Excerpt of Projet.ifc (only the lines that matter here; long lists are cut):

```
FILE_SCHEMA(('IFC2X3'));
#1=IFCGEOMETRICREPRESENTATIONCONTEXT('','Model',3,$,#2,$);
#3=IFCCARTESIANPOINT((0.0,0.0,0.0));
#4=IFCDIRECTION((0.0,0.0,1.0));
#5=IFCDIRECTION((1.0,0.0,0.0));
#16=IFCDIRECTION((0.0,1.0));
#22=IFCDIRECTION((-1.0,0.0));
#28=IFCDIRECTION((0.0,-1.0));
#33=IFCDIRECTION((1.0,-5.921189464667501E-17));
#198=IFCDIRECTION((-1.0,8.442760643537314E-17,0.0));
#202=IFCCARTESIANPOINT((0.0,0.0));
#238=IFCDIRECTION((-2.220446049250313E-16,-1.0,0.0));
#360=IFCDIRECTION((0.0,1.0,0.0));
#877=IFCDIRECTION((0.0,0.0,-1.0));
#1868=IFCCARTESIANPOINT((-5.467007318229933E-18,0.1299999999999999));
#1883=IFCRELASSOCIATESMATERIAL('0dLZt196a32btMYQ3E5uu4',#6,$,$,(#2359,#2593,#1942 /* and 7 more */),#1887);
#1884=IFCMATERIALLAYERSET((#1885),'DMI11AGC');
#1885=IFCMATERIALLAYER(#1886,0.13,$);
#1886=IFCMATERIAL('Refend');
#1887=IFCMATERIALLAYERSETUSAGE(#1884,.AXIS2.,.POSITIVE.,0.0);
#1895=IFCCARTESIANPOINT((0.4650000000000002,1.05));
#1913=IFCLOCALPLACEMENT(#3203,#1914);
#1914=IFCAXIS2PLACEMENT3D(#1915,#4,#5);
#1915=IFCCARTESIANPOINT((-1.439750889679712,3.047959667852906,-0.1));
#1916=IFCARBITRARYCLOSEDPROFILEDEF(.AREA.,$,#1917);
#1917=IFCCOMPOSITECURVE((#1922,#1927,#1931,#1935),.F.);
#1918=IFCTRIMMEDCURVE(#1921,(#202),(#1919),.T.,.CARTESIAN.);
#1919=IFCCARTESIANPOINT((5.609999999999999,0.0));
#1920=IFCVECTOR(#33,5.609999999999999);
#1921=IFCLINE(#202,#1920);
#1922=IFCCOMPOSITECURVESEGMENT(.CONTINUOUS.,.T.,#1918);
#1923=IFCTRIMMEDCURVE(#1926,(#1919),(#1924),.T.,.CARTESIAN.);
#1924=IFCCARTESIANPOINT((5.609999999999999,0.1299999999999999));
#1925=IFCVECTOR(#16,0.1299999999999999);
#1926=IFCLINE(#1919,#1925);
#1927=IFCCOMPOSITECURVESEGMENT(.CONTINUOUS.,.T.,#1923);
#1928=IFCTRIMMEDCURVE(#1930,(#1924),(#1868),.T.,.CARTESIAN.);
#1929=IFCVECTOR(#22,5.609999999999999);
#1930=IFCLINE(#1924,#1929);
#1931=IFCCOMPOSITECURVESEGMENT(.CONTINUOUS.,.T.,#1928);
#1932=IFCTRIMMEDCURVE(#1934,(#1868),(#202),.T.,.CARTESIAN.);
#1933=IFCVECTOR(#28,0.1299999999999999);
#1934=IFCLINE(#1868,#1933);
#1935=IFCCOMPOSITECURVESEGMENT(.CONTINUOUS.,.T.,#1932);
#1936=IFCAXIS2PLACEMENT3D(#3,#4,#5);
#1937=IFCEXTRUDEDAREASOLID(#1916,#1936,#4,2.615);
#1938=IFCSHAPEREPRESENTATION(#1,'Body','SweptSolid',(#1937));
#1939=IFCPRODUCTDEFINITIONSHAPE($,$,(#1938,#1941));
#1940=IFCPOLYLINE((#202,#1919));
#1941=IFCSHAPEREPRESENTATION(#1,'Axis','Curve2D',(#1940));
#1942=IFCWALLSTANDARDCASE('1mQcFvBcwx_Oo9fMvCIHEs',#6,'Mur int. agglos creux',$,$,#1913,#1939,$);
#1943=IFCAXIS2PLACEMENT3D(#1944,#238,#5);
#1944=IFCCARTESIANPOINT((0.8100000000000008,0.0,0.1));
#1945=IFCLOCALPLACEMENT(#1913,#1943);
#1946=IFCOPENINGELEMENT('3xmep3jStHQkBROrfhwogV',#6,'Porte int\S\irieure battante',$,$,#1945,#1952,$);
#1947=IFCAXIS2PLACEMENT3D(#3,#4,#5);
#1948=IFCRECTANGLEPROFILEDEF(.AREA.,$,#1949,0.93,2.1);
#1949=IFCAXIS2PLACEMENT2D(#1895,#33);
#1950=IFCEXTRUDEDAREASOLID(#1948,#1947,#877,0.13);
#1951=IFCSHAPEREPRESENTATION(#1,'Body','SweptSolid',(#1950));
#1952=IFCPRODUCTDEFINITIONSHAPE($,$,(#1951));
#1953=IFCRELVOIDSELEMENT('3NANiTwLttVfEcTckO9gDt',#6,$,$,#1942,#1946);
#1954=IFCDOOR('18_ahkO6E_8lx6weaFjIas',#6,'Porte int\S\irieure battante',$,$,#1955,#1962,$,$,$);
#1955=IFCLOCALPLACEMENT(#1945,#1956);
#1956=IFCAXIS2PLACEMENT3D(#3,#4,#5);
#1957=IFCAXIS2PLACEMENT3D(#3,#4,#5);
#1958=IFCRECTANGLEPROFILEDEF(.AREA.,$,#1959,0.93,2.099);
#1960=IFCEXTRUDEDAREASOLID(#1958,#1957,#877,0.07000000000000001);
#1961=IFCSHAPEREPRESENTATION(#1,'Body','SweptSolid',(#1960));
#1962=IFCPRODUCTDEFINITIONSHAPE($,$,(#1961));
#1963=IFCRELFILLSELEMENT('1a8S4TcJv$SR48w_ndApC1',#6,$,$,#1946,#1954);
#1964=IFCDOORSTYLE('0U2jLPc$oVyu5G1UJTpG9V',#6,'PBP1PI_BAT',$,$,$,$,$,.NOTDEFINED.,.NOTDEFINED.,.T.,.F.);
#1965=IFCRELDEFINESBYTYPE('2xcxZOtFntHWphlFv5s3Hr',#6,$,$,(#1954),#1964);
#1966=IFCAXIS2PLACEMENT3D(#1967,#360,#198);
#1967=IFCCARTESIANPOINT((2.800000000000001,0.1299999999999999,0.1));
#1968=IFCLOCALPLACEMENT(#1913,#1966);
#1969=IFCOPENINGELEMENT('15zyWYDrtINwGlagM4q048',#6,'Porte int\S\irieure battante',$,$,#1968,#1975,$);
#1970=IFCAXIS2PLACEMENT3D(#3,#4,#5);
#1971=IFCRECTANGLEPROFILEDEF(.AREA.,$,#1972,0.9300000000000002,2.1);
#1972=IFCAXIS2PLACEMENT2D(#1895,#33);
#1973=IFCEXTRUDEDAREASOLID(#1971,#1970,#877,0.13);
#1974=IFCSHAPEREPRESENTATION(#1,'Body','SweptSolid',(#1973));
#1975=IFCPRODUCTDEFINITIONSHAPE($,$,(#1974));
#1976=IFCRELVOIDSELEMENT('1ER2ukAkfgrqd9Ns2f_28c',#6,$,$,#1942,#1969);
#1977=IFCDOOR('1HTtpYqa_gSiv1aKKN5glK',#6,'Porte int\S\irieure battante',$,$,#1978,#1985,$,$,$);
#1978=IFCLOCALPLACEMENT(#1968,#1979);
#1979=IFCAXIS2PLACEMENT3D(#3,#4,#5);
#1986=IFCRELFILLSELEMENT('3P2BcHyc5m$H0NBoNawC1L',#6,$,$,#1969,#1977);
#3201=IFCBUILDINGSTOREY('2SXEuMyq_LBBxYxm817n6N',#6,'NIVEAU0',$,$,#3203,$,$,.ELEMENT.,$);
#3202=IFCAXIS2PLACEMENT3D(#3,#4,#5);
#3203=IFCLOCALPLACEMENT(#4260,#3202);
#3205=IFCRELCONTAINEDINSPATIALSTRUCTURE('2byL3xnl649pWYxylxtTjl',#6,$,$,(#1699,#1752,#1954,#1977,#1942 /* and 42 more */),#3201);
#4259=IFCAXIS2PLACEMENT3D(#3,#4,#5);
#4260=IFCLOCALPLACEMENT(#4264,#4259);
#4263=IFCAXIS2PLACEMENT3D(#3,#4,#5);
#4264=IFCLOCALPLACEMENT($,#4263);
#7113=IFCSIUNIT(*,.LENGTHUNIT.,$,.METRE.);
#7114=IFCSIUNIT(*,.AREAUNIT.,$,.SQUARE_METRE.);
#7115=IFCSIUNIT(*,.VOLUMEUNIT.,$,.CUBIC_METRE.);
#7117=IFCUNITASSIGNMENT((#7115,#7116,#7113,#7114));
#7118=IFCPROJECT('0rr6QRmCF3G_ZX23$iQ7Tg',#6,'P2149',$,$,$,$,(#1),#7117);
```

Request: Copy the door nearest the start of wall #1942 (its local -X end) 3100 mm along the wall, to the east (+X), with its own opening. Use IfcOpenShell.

```python
import ifcopenshell
import ifcopenshell.api.feature
import ifcopenshell.api.geometry
import ifcopenshell.api.root
import ifcopenshell.geom
import ifcopenshell.util.element
import ifcopenshell.util.placement
import ifcopenshell.util.shape
import ifcopenshell.util.unit

model = ifcopenshell.open("Projet.ifc")
unit_scale = ifcopenshell.util.unit.calculate_unit_scale(model)
settings = ifcopenshell.geom.settings()


def volume(element):
    """Net volume in cubic metres, openings subtracted."""
    shape = ifcopenshell.geom.create_shape(settings, element)
    return ifcopenshell.util.shape.get_volume(shape.geometry)


door = model.by_guid("18_ahkO6E_8lx6weaFjIas")
opening = door.FillsVoids[0].RelatingOpeningElement
wall = opening.VoidsElements[0].RelatingBuildingElement
before = volume(wall)
shift = ifcopenshell.util.placement.get_local_placement(wall.ObjectPlacement)[:3, 0] * 3.1 / unit_scale

# copy_class copies the void relationship, type, container and properties, but no geometry.
new_opening = ifcopenshell.api.root.copy_class(model, product=opening)
new_opening.Representation = ifcopenshell.util.element.copy_deep(
    model, opening.Representation, exclude=["IfcGeometricRepresentationContext", "IfcRepresentationMap"]
)
new_door = ifcopenshell.api.root.copy_class(model, product=door)
new_door.Representation = ifcopenshell.util.element.copy_deep(
    model, door.Representation, exclude=["IfcGeometricRepresentationContext", "IfcRepresentationMap"]
)
fills = ifcopenshell.api.feature.add_filling(model, opening=new_opening, element=new_door)
fills.OwnerHistory = new_door.OwnerHistory  # required in IFC2X3

for old, new in ((opening, new_opening), (door, new_door)):
    matrix = ifcopenshell.util.placement.get_local_placement(old.ObjectPlacement)
    matrix[:3, 3] += shift
    ifcopenshell.api.geometry.edit_object_placement(model, product=new, matrix=matrix, is_si=False)

after = volume(wall)

print(f"wall volume {before:.3f} -> {after:.3f} m3")

model.write("Projet_rev.ifc")
```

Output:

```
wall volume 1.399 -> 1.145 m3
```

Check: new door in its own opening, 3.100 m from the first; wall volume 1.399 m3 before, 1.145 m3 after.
